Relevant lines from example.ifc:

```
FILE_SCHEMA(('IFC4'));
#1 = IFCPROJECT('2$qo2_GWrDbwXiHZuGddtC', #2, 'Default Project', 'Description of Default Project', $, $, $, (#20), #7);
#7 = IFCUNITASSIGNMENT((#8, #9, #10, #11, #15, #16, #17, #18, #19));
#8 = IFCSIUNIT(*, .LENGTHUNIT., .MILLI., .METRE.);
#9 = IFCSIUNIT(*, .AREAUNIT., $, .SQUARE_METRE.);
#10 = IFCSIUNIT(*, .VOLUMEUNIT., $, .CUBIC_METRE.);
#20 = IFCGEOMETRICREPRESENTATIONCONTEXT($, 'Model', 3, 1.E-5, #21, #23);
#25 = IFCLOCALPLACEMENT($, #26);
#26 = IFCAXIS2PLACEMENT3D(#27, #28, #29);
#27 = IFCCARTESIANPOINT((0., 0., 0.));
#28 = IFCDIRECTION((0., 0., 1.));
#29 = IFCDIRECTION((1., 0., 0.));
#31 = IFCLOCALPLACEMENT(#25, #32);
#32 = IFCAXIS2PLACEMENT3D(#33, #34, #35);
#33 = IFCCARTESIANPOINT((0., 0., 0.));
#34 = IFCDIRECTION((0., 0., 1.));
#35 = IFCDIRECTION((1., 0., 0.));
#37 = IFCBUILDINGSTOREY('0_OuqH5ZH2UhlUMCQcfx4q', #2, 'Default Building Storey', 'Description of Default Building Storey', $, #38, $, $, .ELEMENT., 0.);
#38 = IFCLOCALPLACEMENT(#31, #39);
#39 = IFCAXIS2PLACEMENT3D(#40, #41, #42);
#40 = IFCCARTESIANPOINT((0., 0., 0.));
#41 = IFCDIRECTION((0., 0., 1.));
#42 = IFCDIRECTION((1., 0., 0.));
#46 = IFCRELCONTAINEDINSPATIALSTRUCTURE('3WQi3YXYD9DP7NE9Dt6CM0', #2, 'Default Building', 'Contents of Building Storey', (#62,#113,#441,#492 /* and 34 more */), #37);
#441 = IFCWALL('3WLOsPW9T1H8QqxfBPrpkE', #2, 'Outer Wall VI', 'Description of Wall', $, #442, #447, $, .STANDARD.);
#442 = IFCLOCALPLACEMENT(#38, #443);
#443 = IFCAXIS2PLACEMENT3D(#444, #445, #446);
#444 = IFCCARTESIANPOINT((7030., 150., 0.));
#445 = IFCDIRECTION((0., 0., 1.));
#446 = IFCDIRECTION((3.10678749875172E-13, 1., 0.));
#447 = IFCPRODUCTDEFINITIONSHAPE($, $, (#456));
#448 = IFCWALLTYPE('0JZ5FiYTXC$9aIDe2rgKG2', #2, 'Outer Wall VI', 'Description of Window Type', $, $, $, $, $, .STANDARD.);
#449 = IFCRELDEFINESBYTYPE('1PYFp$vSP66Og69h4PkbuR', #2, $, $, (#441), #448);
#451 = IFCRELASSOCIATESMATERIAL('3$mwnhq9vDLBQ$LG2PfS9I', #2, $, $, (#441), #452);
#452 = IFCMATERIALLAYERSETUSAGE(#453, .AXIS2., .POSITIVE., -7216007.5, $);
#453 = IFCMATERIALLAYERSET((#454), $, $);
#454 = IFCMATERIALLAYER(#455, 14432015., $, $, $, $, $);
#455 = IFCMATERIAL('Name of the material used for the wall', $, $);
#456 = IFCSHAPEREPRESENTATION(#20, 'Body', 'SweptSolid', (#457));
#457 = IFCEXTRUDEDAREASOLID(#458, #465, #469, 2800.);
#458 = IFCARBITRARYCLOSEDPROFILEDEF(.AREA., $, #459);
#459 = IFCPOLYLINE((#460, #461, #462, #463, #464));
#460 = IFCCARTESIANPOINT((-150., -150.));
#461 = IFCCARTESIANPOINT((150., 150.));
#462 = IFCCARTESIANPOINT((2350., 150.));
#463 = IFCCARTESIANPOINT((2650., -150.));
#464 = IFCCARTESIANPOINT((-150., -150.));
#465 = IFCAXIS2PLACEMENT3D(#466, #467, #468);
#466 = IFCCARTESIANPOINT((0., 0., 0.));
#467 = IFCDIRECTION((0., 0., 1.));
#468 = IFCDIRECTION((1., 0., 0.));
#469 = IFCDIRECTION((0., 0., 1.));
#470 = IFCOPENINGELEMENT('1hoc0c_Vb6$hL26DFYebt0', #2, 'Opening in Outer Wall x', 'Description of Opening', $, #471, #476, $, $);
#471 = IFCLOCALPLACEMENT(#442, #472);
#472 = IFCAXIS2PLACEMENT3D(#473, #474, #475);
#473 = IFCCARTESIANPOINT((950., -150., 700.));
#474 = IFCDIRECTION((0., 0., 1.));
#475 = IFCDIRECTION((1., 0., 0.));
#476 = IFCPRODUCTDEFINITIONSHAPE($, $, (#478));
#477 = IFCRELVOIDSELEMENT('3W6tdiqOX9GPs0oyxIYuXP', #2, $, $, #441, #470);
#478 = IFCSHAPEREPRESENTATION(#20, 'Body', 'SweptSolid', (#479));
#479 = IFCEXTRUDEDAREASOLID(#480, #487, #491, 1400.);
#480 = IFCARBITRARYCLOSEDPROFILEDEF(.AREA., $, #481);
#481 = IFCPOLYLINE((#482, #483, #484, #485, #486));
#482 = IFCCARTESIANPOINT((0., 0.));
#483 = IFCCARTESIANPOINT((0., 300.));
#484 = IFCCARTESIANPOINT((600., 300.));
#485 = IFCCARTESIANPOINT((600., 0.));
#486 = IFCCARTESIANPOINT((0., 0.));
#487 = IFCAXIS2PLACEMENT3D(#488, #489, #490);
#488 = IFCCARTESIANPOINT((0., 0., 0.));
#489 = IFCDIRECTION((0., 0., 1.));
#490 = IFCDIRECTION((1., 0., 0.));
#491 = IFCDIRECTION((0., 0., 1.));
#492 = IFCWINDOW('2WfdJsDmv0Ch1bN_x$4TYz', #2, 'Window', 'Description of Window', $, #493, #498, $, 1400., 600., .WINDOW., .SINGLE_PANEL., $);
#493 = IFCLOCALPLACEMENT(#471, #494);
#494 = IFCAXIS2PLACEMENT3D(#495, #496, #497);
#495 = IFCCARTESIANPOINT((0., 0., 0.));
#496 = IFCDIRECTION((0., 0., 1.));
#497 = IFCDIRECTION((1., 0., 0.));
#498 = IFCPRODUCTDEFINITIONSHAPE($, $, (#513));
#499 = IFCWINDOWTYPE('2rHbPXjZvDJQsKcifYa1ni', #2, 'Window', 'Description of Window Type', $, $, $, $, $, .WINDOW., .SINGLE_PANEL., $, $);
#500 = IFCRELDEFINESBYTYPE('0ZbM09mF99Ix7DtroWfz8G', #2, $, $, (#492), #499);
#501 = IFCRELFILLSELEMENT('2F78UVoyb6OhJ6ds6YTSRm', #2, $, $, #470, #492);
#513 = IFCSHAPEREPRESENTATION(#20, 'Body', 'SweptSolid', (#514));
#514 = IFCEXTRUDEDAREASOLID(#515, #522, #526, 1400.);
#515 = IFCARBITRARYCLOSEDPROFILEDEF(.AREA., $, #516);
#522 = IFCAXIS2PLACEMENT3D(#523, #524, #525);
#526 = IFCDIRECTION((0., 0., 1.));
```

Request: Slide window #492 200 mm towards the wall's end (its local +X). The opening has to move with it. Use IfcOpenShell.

```python
import ifcopenshell
import ifcopenshell.api.geometry
import ifcopenshell.util.placement

model = ifcopenshell.open("example.ifc")

window = model.by_guid("2WfdJsDmv0Ch1bN_x$4TYz")
opening = window.FillsVoids[0].RelatingOpeningElement
wall = opening.VoidsElements[0].RelatingBuildingElement

wall_matrix = ifcopenshell.util.placement.get_local_placement(wall.ObjectPlacement)
shift = wall_matrix[:3, 0] * 200.0
before = ifcopenshell.util.placement.get_local_placement(window.ObjectPlacement)[:3, 3].copy()

# The window is placed relative to its opening, so it follows when the opening moves.
matrix = ifcopenshell.util.placement.get_local_placement(opening.ObjectPlacement)
matrix[:3, 3] += shift
ifcopenshell.api.geometry.edit_object_placement(
    model, product=opening, matrix=matrix, is_si=False, should_transform_children=True
)

after = ifcopenshell.util.placement.get_local_placement(window.ObjectPlacement)[:3, 3]
print("window moved by", (after - before).round(3) + 0.0)

model.write("example_v2.ifc")
```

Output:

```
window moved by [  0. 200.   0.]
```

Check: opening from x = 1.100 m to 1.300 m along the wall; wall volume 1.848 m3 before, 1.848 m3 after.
